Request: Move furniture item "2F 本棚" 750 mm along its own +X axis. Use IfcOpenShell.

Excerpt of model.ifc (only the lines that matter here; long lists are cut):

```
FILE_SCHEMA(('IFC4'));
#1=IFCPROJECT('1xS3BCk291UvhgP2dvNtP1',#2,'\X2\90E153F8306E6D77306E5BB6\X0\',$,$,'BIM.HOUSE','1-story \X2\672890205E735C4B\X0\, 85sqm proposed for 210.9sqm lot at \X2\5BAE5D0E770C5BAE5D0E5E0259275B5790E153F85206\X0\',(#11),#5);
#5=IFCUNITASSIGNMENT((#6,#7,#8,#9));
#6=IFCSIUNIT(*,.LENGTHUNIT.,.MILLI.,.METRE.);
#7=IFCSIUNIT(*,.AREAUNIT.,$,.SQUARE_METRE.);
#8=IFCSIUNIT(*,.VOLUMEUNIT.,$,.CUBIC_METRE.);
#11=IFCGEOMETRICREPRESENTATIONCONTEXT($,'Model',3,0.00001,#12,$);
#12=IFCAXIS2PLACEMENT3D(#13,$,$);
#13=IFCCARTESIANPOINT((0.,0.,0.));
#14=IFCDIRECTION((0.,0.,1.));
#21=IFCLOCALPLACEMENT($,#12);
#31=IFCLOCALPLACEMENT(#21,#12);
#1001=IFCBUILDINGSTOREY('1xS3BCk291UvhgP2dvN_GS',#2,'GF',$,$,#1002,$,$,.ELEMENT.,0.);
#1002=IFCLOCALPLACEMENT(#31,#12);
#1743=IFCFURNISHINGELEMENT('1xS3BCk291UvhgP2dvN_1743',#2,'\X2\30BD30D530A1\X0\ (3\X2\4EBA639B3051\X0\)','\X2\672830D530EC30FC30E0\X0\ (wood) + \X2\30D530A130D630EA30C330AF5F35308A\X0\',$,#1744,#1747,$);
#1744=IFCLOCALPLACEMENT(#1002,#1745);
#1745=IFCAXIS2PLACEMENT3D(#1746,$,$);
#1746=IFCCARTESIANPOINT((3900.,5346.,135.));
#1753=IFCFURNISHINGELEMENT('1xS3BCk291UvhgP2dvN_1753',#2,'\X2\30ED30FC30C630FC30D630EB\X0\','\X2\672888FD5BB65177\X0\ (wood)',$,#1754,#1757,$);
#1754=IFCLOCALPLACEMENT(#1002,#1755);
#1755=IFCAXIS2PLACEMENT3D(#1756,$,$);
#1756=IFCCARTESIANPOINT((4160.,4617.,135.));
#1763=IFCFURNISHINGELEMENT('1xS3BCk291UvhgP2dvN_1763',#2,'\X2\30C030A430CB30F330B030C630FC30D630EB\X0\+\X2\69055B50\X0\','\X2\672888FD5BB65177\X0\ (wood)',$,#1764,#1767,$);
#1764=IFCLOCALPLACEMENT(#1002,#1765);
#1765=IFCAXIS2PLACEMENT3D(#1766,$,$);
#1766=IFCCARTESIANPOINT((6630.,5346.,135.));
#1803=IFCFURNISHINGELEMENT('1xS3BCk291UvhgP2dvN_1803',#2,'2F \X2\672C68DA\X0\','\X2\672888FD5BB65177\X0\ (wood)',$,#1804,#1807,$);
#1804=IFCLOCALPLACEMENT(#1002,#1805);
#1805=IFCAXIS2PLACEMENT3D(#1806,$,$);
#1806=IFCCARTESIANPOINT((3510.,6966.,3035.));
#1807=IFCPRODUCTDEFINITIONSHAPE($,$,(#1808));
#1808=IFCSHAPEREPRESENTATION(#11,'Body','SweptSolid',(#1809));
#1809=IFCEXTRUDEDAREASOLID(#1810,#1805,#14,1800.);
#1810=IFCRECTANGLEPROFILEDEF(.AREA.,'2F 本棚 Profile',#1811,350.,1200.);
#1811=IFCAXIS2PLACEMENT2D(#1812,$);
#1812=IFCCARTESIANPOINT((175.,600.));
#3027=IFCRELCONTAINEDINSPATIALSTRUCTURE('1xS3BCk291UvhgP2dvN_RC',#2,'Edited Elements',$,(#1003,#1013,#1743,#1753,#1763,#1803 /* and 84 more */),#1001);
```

```python
import ifcopenshell
import ifcopenshell.api.geometry
import ifcopenshell.util.placement
import ifcopenshell.util.unit

model = ifcopenshell.open("model.ifc")
unit_scale = ifcopenshell.util.unit.calculate_unit_scale(model)

item = model.by_guid("1xS3BCk291UvhgP2dvN_1803")
matrix = ifcopenshell.util.placement.get_local_placement(item.ObjectPlacement)
matrix[:3, 3] += matrix[:3, 0] * 0.75 / unit_scale
ifcopenshell.api.geometry.edit_object_placement(model, product=item, matrix=matrix, is_si=False)

print(ifcopenshell.util.placement.get_local_placement(item.ObjectPlacement).round(3) + 0.0)

model.write("model_v2.ifc")
```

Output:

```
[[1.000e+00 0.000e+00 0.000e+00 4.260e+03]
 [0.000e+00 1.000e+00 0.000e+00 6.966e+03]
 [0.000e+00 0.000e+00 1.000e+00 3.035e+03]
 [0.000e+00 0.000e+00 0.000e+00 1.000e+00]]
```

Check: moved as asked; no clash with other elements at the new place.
